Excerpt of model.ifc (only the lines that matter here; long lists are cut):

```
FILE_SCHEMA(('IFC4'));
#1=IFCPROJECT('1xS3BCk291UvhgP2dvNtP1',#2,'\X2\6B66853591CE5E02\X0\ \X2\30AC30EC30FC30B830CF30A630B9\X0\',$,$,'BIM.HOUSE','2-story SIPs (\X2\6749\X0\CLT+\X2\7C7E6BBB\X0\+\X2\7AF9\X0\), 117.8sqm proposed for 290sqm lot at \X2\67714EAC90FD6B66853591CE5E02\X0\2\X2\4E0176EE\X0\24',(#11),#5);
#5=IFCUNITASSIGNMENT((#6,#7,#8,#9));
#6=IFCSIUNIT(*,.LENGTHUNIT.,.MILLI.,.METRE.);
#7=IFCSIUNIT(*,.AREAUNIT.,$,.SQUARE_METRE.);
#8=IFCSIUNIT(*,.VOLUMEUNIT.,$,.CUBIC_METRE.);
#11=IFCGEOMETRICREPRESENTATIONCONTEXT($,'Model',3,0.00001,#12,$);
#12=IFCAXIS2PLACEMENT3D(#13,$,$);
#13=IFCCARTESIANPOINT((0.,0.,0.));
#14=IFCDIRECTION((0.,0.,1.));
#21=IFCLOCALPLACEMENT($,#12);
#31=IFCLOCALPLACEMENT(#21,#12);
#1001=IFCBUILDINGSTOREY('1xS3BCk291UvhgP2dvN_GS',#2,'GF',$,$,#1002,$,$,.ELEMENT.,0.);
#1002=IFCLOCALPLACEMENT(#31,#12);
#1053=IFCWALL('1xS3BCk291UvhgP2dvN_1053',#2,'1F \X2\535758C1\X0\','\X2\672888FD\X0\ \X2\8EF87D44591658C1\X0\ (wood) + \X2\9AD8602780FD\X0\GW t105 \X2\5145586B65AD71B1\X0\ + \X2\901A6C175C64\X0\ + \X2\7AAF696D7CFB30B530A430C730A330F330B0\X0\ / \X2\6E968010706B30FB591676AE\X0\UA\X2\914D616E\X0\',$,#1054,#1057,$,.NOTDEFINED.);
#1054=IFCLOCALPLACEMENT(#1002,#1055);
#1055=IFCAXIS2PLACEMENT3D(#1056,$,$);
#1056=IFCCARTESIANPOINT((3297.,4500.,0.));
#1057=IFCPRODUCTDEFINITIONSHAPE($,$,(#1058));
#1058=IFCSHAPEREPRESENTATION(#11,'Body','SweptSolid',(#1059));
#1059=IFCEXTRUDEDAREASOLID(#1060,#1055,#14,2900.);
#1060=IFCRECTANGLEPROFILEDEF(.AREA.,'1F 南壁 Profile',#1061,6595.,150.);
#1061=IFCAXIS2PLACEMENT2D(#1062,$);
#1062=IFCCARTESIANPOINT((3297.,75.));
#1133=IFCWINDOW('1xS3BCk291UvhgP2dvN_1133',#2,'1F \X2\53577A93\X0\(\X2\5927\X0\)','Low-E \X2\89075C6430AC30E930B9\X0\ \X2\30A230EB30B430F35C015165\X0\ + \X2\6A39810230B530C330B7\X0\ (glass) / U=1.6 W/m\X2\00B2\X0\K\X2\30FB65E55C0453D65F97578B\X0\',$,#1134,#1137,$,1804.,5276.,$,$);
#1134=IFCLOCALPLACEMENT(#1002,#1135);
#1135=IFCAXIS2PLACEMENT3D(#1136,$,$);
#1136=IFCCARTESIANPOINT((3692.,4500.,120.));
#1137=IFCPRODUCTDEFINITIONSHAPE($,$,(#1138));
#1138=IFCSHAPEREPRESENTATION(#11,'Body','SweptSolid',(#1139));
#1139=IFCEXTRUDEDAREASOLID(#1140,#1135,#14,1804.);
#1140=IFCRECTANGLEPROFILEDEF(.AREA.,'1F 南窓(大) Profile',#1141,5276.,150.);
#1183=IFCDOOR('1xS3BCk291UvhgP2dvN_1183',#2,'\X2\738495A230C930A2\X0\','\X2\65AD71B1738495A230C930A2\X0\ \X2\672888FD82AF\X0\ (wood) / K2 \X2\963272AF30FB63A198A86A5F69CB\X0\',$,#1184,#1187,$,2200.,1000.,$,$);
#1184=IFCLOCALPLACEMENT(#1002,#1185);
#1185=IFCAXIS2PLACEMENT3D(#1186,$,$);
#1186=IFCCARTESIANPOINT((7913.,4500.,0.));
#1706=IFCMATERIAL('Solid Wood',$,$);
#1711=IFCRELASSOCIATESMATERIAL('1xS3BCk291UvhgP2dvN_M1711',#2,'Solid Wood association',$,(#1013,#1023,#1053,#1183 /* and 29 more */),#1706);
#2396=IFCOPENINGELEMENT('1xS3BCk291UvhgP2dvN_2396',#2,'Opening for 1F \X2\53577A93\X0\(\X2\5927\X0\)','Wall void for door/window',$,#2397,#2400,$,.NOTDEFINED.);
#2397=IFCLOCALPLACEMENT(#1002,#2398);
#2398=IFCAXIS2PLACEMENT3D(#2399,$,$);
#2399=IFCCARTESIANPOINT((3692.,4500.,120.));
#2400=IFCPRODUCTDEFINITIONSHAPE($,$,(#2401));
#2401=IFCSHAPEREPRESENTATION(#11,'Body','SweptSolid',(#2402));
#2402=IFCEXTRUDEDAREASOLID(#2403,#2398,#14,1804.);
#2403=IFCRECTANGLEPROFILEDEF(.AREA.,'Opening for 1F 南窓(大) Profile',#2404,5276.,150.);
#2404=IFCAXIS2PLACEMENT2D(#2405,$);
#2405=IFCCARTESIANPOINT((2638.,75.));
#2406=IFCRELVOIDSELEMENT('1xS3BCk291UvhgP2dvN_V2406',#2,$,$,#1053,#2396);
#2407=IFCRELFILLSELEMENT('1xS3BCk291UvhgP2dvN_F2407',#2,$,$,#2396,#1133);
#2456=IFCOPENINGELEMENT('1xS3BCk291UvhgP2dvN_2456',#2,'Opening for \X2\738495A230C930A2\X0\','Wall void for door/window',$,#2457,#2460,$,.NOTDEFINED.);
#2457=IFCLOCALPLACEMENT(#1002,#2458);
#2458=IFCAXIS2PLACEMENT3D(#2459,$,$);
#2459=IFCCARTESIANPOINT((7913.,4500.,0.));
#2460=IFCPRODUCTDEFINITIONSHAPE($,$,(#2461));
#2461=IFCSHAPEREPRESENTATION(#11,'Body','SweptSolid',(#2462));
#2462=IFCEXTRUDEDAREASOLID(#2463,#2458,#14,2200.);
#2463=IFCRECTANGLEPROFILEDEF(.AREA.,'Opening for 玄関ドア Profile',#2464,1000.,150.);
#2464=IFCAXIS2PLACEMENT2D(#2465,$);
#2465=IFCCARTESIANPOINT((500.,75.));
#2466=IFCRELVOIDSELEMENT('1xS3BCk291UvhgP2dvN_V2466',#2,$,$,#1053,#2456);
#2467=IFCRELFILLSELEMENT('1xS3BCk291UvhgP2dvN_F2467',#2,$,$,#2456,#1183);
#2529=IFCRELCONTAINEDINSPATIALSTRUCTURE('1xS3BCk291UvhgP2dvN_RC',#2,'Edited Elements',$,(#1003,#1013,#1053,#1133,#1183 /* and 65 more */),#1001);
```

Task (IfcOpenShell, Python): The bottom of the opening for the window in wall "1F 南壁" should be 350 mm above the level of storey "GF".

```python
import numpy as np
import ifcopenshell
import ifcopenshell.api.geometry
import ifcopenshell.geom
import ifcopenshell.util.element
import ifcopenshell.util.placement
import ifcopenshell.util.shape
import ifcopenshell.util.unit

model = ifcopenshell.open("model.ifc")
unit_scale = ifcopenshell.util.unit.calculate_unit_scale(model)

window = model.by_guid("1xS3BCk291UvhgP2dvN_1133")
opening = window.FillsVoids[0].RelatingOpeningElement
storey = ifcopenshell.util.element.get_container(window, ifc_class="IfcBuildingStorey")
level = ifcopenshell.util.placement.get_local_placement(storey.ObjectPlacement)[2, 3]

# The opening's origin need not be at the sill, so measure its lowest point.
shape = ifcopenshell.geom.create_shape(ifcopenshell.geom.settings(), opening)
bottom = ifcopenshell.util.shape.get_shape_bottom_elevation(shape, shape.geometry) / unit_scale
dz = level + 350.0 - bottom

shift = np.array([0.0, 0.0, dz])
# The window is not placed relative to its opening, so move both.
for product in (opening, window):
    matrix = ifcopenshell.util.placement.get_local_placement(product.ObjectPlacement)
    matrix[:3, 3] += shift
    ifcopenshell.api.geometry.edit_object_placement(model, product=product, matrix=matrix, is_si=False)

print(f"moved by {dz * unit_scale:+.3f} m")

model.write("model-out.ifc")
```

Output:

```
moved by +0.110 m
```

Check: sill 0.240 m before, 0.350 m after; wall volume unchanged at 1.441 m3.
